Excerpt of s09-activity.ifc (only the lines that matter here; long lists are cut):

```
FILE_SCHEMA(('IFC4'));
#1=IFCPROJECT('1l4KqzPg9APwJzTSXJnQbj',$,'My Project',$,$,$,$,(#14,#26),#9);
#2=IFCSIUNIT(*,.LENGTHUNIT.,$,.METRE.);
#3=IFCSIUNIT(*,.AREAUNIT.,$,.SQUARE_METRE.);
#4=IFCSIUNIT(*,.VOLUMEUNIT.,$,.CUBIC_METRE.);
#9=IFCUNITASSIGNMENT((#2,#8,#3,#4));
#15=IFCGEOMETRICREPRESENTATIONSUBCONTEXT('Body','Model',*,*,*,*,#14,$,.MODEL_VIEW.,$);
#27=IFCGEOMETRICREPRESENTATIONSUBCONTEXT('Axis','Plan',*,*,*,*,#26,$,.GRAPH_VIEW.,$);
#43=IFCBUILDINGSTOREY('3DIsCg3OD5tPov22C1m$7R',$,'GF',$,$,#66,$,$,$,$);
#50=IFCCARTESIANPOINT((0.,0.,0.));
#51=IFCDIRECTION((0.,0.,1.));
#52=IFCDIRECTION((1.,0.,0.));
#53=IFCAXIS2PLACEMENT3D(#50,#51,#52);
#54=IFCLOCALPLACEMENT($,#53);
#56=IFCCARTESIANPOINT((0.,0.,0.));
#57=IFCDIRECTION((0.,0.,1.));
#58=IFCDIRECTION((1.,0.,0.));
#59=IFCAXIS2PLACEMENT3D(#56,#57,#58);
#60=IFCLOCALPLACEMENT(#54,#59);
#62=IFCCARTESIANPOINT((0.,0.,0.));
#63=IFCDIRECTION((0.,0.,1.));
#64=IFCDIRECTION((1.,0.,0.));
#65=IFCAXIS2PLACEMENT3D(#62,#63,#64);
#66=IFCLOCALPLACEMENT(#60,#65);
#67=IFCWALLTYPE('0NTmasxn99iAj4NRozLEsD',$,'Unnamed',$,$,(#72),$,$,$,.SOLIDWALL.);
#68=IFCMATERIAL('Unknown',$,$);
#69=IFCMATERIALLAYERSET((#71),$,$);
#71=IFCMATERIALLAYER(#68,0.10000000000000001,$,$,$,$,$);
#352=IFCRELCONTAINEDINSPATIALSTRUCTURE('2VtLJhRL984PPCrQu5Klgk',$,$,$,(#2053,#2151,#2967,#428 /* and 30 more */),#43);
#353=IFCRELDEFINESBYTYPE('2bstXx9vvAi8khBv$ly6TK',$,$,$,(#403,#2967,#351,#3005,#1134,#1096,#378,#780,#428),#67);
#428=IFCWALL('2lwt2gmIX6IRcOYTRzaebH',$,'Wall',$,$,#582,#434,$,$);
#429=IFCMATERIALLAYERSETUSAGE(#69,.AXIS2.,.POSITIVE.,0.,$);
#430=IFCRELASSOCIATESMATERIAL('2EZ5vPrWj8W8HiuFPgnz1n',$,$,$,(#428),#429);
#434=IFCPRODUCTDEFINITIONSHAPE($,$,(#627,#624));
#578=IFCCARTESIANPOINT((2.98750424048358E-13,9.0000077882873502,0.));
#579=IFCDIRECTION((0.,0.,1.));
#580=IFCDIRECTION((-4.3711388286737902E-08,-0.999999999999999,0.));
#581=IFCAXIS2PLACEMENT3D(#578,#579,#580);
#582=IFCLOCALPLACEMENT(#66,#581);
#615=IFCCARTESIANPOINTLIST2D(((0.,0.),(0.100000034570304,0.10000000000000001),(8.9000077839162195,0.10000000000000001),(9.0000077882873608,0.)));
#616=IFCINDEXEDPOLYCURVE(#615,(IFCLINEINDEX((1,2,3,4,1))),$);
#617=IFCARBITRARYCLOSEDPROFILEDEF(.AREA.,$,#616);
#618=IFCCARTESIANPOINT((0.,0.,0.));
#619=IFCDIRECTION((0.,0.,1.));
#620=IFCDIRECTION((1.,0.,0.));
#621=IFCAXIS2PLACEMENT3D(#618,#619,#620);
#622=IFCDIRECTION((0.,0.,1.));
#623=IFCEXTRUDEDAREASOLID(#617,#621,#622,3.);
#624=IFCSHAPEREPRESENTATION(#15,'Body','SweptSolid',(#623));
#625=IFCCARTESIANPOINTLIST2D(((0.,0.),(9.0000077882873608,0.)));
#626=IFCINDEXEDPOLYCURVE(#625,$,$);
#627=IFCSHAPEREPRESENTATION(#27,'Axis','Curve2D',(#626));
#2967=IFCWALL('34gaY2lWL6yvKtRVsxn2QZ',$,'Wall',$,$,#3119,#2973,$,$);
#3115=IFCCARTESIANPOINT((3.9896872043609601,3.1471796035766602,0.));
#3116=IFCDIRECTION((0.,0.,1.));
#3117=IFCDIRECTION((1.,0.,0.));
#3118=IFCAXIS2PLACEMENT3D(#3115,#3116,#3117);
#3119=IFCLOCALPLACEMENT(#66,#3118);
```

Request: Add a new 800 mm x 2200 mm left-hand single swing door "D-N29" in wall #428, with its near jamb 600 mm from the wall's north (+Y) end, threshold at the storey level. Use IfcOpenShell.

```python
import numpy as np
import ifcopenshell
import ifcopenshell.api.feature
import ifcopenshell.api.geometry
import ifcopenshell.api.root
import ifcopenshell.api.spatial
import ifcopenshell.geom
import ifcopenshell.util.element
import ifcopenshell.util.placement
import ifcopenshell.util.representation
import ifcopenshell.util.shape
import ifcopenshell.util.unit

model = ifcopenshell.open("s09-activity.ifc")
unit_scale = ifcopenshell.util.unit.calculate_unit_scale(model)
settings = ifcopenshell.geom.settings()


def volume(element):
    """Net volume in cubic metres, openings subtracted."""
    shape = ifcopenshell.geom.create_shape(settings, element)
    return ifcopenshell.util.shape.get_volume(shape.geometry)


wall = model.by_guid("2lwt2gmIX6IRcOYTRzaebH")
storey = ifcopenshell.util.element.get_container(wall, ifc_class="IfcBuildingStorey")
context = ifcopenshell.util.representation.get_context(model, "Model", "Body", "MODEL_VIEW")
before = volume(wall)

width, height, from_end, sill = 0.8, 2.2, 0.6, 0.0  # metres

# The wall runs along its own X axis, and the end named is its -X end.
wall_shape = ifcopenshell.geom.create_shape(settings, wall)
x, y, z = ifcopenshell.util.shape.get_vertices(wall_shape.geometry).T
start = x.min() + from_end
face, thickness = float(y.min()), float(y.max() - y.min())
wall_matrix = ifcopenshell.util.placement.get_local_placement(wall.ObjectPlacement)
level = ifcopenshell.util.placement.get_local_placement(storey.ObjectPlacement)[2, 3]


def in_wall(x, y):
    """Placement at x, y metres in the wall's axes, at sill height."""
    matrix = wall_matrix.copy()
    matrix[:, 3] = wall_matrix @ np.array([x / unit_scale, y / unit_scale, 0.0, 1.0])
    matrix[2, 3] = level + sill / unit_scale
    return matrix


# Opening: a box that overshoots both wall faces by 50 mm.
opening = ifcopenshell.api.root.create_entity(model, ifc_class="IfcOpeningElement", predefined_type="OPENING")
box = ifcopenshell.api.geometry.add_wall_representation(
    model, context=context, length=width, height=height, thickness=thickness + 0.1
)
ifcopenshell.api.geometry.assign_representation(model, product=opening, representation=box)
ifcopenshell.api.geometry.edit_object_placement(model, product=opening, matrix=in_wall(start, face - 0.05), is_si=False)
ifcopenshell.api.feature.add_feature(model, feature=opening, element=wall)

door = ifcopenshell.api.root.create_entity(model, ifc_class="IfcDoor", name="D-N29", predefined_type="DOOR")
door.OverallWidth, door.OverallHeight = width / unit_scale, height / unit_scale
door.OperationType = "SINGLE_SWING_LEFT"
body = ifcopenshell.api.geometry.add_door_representation(
    model,
    context=context,
    overall_width=door.OverallWidth,
    overall_height=door.OverallHeight,
    operation_type="SINGLE_SWING_LEFT",
    lining_properties={"LiningDepth": thickness / unit_scale, "ThresholdDepth": thickness / unit_scale},
)
ifcopenshell.api.geometry.assign_representation(model, product=door, representation=body)
ifcopenshell.api.spatial.assign_container(model, products=[door], relating_structure=storey)
ifcopenshell.api.feature.add_filling(model, opening=opening, element=door)

# The lining spans the wall, so the door starts at the wall face.
ifcopenshell.api.geometry.edit_object_placement(model, product=door, matrix=in_wall(start, face), is_si=False)

after = volume(wall)

print(f"wall volume {before:.3f} -> {after:.3f} m3")

model.write("s09-activity_updated.ifc")
```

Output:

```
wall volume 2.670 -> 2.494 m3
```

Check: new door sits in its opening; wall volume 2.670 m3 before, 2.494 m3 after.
